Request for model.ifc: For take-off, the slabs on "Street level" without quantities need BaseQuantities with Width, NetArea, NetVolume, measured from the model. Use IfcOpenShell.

First a look at what the model holds.

```python
import ifcopenshell
import ifcopenshell.util.element
import ifcopenshell.util.unit

model = ifcopenshell.open("model.ifc")
print(model.schema)
for unit_type in ("LENGTHUNIT", "AREAUNIT", "VOLUMEUNIT"):
    print(unit_type, ifcopenshell.util.unit.calculate_unit_scale(model, unit_type))
storey = next(s for s in model.by_type("IfcBuildingStorey") if s.Name == "Street level")
slabs = [e for e in ifcopenshell.util.element.get_decomposition(storey) if e.is_a("IfcSlab")]
for e in sorted(slabs, key=lambda e: e.id()):
    print(e.id(), e.is_a(), e.Name, list(ifcopenshell.util.element.get_psets(e, qtos_only=True)), sep=" | ")
```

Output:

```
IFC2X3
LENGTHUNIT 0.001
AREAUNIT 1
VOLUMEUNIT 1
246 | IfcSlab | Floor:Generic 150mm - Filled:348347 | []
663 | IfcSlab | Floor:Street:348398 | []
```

```python
import ifcopenshell
import ifcopenshell.api.pset
import ifcopenshell.geom
import ifcopenshell.util.element
import ifcopenshell.util.shape
import ifcopenshell.util.unit

model = ifcopenshell.open("model.ifc")
unit_scale = ifcopenshell.util.unit.calculate_unit_scale(model)
area_scale = ifcopenshell.util.unit.calculate_unit_scale(model, "AREAUNIT")
volume_scale = ifcopenshell.util.unit.calculate_unit_scale(model, "VOLUMEUNIT")
settings = ifcopenshell.geom.settings()

storey = next(s for s in model.by_type("IfcBuildingStorey") if s.Name == "Street level")
slabs = [e for e in ifcopenshell.util.element.get_decomposition(storey) if e.is_a("IfcSlab")]

for e in sorted(slabs, key=lambda e: e.id()):
    if ifcopenshell.util.element.get_psets(e, qtos_only=True, should_inherit=False):
        continue
    # Geometry comes back in metres, in the element's own axes.
    shape = ifcopenshell.geom.create_shape(settings, e)
    values = {
        "Width": ifcopenshell.util.shape.get_z(shape.geometry) / unit_scale,
        "NetArea": ifcopenshell.util.shape.get_footprint_area(shape.geometry) / area_scale,
        "NetVolume": ifcopenshell.util.shape.get_volume(shape.geometry) / volume_scale,
    }
    qto = ifcopenshell.api.pset.add_qto(model, product=e, name="BaseQuantities")
    ifcopenshell.api.pset.edit_qto(model, qto=qto, properties=values)
    print(e.id(), {k: round(v, 3) for k, v in values.items()})

model.write("model-out.ifc")
```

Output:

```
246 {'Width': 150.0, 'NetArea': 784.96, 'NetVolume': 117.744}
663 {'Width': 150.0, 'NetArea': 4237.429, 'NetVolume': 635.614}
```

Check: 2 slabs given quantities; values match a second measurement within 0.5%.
